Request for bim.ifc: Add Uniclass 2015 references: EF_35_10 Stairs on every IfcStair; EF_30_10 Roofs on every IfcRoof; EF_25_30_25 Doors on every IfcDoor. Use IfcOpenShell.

First a look at what the model holds.

```python
import ifcopenshell

model = ifcopenshell.open("bim.ifc")
print(model.schema)
print("classifications:", [c.Name for c in model.by_type("IfcClassification")])
for ifc_class in ("IfcDoor", "IfcRoof", "IfcStair", "IfcWall", "IfcWindow"):
    print(ifc_class, len(model.by_type(ifc_class)))
```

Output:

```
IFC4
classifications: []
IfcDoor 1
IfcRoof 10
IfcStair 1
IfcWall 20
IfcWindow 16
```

```python
import ifcopenshell
import ifcopenshell.api.classification

model = ifcopenshell.open("bim.ifc")

system = ifcopenshell.api.classification.add_classification(model, classification="Uniclass 2015")

codes = {
    "IfcStair": ("EF_35_10", "Stairs"),
    "IfcRoof": ("EF_30_10", "Roofs"),
    "IfcDoor": ("EF_25_30_25", "Doors"),
}
for ifc_class, (code, name) in codes.items():
    products = model.by_type(ifc_class)
    ifcopenshell.api.classification.add_reference(
        model, products=products, classification=system, identification=code, name=name
    )
    print(code, len(products))

model.write("bim_edited.ifc")
```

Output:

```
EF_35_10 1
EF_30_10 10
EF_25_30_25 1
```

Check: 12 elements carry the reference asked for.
